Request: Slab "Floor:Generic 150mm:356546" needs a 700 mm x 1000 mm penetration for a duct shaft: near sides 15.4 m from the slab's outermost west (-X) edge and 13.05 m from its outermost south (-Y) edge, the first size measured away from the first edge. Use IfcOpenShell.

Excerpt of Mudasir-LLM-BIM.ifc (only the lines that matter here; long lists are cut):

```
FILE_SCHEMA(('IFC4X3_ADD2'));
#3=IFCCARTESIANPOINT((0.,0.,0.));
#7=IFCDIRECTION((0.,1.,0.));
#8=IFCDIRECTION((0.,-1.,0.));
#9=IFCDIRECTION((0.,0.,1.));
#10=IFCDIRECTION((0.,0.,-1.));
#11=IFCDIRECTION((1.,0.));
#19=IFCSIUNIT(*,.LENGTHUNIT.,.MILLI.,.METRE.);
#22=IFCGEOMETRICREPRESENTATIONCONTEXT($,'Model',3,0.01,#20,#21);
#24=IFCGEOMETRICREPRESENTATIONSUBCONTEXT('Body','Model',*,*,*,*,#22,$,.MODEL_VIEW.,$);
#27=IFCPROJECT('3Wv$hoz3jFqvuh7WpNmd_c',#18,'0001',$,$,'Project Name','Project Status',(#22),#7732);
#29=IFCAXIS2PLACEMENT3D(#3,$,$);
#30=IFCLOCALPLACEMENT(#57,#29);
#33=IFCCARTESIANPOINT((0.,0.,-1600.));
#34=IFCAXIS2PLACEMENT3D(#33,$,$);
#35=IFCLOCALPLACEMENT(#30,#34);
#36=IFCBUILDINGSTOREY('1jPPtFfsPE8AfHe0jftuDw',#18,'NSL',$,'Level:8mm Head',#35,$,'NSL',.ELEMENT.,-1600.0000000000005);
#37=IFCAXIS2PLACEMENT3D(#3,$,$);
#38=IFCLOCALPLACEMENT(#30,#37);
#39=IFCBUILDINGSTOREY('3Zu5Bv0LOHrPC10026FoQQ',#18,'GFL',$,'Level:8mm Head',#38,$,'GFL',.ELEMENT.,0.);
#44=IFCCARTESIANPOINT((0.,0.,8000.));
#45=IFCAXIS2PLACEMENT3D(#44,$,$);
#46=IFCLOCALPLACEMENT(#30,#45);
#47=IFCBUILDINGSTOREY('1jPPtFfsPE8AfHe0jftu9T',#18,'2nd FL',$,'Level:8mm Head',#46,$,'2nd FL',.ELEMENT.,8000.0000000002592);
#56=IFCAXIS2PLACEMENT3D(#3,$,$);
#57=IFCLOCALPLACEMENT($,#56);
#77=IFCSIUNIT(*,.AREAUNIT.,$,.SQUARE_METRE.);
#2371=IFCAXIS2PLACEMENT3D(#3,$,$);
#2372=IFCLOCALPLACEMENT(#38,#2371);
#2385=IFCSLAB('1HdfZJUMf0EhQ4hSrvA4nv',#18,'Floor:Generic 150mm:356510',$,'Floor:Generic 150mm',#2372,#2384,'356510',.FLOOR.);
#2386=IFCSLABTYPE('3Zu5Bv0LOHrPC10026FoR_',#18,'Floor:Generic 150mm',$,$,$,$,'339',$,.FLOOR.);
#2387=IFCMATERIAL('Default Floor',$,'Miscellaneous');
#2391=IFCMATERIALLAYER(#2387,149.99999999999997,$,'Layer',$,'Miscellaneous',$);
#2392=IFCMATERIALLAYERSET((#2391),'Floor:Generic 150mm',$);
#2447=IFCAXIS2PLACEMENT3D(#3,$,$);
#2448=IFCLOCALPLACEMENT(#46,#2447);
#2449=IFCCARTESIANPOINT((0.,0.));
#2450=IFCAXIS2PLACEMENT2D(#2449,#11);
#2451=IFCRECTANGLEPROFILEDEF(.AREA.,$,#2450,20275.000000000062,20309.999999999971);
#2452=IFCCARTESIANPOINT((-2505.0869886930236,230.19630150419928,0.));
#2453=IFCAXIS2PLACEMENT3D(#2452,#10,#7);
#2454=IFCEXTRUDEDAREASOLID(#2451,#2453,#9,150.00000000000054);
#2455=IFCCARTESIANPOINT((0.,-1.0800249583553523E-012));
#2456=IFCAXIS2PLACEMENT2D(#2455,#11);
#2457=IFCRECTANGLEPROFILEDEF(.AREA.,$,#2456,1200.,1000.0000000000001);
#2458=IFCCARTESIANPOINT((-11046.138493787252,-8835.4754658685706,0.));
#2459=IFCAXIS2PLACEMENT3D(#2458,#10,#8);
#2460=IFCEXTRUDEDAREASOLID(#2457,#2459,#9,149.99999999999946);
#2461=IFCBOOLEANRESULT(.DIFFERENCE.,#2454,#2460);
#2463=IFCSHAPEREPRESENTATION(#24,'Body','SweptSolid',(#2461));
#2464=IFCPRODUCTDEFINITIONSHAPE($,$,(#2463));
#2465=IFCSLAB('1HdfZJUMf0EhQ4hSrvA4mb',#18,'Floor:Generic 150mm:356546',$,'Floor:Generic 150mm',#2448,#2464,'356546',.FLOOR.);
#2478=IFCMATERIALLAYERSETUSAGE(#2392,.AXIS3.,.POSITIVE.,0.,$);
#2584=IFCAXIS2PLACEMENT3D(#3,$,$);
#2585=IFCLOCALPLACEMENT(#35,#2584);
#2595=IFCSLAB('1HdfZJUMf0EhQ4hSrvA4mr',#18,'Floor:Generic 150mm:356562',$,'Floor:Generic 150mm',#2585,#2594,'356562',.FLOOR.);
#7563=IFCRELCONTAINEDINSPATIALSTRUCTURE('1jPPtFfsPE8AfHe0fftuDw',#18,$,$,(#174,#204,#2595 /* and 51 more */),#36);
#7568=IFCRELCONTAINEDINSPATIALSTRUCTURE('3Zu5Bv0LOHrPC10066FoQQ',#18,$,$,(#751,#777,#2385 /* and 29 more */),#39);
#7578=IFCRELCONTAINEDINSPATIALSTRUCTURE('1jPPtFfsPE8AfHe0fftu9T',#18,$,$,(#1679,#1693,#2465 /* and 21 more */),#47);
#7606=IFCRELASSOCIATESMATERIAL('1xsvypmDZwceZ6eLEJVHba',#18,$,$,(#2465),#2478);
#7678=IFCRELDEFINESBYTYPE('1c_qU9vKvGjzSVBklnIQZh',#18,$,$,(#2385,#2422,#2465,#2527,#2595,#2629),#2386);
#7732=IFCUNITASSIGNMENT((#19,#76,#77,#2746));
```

```python
import numpy as np
import ifcopenshell
import ifcopenshell.api.feature
import ifcopenshell.api.geometry
import ifcopenshell.api.root
import ifcopenshell.geom
import ifcopenshell.util.placement
import ifcopenshell.util.representation
import ifcopenshell.util.shape
import ifcopenshell.util.unit

model = ifcopenshell.open("Mudasir-LLM-BIM.ifc")
unit_scale = ifcopenshell.util.unit.calculate_unit_scale(model)
settings = ifcopenshell.geom.settings()


def volume(element):
    """Net volume in cubic metres, openings subtracted."""
    shape = ifcopenshell.geom.create_shape(settings, element)
    return ifcopenshell.util.shape.get_volume(shape.geometry)


slab = model.by_guid("1HdfZJUMf0EhQ4hSrvA4mb")
before = volume(slab)

# Extent in the slab's own axes, in metres. The edges named are its -X and -Y sides.
slab_shape = ifcopenshell.geom.create_shape(settings, slab)
vertices = ifcopenshell.util.shape.get_vertices(slab_shape.geometry)
x_min, y_min, bottom = vertices.min(axis=0)
top = vertices[:, 2].max()

opening = ifcopenshell.api.root.create_entity(model, ifc_class="IfcOpeningElement", name="Duct shaft opening", predefined_type="OPENING")
context = ifcopenshell.util.representation.get_context(model, "Model", "Body", "MODEL_VIEW")
width, depth = 0.7, 1
outline = [(0.0, 0.0), (width, 0.0), (width, depth), (0.0, depth), (0.0, 0.0)]
# Overshoot both faces by 50 mm so the cut is clean.
shape = ifcopenshell.api.geometry.add_slab_representation(
    model, context=context, depth=top - bottom + 0.1, polyline=outline
)
ifcopenshell.api.geometry.assign_representation(model, product=opening, representation=shape)

matrix = ifcopenshell.util.placement.get_local_placement(slab.ObjectPlacement)
matrix[:, 3] = matrix @ np.append(np.array([x_min + 15.4, y_min + 13.05, bottom - 0.05]) / unit_scale, 1.0)
ifcopenshell.api.geometry.edit_object_placement(model, product=opening, matrix=matrix, is_si=False)
ifcopenshell.api.feature.add_feature(model, feature=opening, element=slab)

after = volume(slab)

print(f"slab volume {before:.3f} -> {after:.3f} m3")

model.write("Mudasir-LLM-BIM_updated.ifc")
```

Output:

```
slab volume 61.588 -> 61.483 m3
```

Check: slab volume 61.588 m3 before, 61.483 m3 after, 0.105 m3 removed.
